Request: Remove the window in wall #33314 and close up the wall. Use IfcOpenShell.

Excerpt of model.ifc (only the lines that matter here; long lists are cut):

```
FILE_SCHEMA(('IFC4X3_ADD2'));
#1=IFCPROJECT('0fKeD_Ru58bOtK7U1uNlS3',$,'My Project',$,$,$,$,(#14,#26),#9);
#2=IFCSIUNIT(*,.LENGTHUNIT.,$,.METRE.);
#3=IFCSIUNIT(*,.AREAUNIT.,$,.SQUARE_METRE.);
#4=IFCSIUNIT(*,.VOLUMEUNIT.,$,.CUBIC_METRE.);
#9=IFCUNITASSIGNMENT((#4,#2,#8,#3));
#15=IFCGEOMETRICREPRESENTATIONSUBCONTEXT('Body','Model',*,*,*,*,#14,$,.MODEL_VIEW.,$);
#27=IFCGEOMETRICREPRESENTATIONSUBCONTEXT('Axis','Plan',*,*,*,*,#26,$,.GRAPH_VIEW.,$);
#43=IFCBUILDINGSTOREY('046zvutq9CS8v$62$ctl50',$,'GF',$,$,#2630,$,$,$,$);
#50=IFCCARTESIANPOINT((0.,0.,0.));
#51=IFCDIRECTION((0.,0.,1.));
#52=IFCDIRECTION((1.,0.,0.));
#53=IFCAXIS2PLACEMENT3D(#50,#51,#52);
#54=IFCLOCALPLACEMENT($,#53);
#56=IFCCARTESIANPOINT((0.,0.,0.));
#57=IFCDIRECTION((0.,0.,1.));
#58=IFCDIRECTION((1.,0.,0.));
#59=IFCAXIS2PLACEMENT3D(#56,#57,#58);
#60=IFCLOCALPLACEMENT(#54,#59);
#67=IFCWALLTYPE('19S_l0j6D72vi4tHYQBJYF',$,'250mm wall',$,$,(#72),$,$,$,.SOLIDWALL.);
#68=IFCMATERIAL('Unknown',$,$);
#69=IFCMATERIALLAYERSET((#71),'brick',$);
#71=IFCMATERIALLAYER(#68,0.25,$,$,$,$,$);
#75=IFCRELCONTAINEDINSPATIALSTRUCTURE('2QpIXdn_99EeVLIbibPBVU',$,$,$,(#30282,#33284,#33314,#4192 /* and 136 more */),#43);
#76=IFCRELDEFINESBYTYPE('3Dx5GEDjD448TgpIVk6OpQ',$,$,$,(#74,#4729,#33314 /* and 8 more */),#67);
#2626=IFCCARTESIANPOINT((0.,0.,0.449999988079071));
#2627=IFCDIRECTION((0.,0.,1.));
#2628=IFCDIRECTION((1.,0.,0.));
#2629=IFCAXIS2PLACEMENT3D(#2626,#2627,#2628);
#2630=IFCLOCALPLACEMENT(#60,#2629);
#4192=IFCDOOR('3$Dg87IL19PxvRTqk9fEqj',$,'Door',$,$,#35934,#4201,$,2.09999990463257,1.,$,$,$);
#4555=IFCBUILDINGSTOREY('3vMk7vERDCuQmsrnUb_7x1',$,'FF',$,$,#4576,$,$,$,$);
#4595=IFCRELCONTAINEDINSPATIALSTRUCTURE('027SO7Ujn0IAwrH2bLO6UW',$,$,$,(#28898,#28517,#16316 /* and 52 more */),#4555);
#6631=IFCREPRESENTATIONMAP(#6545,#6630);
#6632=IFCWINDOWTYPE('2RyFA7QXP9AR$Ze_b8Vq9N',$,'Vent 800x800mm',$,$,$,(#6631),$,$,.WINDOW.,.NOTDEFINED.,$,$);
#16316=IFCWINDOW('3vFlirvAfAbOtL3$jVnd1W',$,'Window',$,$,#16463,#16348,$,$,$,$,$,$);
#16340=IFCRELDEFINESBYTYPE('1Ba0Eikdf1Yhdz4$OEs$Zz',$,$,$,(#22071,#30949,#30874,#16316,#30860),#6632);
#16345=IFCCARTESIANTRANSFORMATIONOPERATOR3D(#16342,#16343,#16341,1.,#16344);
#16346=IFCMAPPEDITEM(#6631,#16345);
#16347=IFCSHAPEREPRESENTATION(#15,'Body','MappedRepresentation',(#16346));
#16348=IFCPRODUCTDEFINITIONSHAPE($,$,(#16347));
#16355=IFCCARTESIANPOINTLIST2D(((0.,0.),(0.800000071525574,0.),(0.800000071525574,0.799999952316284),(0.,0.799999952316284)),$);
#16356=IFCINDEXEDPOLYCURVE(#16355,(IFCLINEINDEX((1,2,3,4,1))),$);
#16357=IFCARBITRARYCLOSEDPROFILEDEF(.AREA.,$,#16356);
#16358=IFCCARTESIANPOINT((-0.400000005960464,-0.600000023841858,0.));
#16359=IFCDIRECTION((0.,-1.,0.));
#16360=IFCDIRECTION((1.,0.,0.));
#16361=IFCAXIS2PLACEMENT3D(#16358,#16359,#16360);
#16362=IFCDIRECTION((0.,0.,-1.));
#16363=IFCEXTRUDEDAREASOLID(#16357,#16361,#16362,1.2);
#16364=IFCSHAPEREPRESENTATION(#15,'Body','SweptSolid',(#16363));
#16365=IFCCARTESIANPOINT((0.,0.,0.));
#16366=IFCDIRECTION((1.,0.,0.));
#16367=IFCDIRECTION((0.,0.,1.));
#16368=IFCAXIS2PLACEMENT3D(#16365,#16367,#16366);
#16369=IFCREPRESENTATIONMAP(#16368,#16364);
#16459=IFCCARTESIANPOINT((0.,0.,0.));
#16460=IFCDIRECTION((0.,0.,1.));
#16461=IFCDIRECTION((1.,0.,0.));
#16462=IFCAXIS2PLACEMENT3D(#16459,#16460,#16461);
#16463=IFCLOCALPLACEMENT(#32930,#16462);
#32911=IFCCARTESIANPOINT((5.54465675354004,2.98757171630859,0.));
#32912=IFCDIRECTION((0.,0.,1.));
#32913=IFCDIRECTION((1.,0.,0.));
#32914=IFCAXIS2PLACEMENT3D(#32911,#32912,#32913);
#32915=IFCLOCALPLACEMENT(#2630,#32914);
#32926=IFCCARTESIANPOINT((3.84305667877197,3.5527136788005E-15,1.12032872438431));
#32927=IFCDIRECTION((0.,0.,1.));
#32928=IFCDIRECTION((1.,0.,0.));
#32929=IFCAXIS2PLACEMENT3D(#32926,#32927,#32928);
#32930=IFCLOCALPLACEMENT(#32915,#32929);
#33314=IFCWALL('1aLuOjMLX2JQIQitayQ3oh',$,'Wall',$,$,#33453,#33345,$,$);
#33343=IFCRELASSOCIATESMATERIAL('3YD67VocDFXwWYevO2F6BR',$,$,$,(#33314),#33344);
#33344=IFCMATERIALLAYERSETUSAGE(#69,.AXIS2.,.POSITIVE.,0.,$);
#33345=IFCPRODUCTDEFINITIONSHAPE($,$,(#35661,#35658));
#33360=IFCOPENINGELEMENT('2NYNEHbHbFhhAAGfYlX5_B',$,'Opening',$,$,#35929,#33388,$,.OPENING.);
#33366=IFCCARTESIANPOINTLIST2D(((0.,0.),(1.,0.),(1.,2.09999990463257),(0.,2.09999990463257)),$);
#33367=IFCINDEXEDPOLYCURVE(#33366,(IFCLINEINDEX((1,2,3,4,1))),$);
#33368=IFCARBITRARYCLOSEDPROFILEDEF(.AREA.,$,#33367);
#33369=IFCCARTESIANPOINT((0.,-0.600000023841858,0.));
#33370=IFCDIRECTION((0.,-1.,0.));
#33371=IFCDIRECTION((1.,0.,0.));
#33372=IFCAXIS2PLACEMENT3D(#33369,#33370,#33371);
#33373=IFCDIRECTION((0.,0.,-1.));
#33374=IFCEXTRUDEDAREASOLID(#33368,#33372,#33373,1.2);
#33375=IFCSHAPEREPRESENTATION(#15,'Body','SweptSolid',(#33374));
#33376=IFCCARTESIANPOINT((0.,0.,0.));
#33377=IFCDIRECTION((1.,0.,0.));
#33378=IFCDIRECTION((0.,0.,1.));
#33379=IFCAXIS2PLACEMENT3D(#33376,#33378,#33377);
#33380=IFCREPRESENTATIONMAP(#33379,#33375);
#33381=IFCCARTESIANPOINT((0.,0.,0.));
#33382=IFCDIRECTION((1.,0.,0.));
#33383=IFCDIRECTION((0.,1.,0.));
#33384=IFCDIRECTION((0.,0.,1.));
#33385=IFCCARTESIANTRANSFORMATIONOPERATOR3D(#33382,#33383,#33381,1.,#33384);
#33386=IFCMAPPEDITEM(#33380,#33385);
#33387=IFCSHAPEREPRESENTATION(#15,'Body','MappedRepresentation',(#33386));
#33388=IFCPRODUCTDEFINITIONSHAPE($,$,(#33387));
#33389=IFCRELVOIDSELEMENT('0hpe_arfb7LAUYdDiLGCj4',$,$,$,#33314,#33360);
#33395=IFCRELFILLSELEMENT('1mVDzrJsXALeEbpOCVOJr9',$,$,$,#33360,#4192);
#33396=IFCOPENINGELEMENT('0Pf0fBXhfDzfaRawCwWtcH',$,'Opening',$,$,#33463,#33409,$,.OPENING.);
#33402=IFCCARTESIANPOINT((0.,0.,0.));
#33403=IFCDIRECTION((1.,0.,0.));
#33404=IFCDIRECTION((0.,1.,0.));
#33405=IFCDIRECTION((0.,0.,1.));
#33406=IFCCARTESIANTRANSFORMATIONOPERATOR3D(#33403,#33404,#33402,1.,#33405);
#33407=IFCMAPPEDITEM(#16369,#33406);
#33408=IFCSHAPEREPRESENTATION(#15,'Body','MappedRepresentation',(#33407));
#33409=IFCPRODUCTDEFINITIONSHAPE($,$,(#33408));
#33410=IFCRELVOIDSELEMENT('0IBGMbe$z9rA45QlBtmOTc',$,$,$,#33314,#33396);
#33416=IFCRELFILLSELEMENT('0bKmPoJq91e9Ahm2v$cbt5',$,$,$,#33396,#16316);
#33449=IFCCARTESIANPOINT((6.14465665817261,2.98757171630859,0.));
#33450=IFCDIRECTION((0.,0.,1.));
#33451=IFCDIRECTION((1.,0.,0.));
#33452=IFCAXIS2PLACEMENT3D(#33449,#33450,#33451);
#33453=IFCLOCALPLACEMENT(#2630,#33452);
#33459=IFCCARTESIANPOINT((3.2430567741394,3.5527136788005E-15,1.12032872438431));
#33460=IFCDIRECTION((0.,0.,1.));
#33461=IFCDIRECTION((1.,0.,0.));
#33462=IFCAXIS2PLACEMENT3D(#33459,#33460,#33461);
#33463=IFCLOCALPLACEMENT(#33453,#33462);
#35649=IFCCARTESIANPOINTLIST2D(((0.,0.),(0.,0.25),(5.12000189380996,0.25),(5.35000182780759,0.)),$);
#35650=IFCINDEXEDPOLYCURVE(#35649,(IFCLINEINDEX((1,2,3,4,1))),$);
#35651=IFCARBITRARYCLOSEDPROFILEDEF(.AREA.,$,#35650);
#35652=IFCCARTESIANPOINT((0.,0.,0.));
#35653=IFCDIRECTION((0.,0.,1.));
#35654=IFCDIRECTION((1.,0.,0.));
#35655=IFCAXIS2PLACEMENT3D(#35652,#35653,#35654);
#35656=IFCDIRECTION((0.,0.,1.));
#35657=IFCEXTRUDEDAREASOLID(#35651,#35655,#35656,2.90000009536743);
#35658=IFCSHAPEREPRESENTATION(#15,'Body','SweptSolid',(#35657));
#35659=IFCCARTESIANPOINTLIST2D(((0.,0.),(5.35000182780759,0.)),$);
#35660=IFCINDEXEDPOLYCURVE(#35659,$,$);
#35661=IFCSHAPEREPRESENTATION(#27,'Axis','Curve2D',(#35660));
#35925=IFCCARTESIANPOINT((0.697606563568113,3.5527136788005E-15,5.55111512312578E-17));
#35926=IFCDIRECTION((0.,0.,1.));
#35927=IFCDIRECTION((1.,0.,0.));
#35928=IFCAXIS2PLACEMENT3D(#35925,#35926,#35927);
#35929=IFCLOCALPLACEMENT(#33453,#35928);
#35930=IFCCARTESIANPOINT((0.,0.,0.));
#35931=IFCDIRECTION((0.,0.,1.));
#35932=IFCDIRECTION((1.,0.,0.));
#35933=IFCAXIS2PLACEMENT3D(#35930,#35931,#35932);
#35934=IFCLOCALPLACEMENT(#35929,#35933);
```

```python
import ifcopenshell
import ifcopenshell.api.feature
import ifcopenshell.api.root
import ifcopenshell.geom
import ifcopenshell.util.shape

model = ifcopenshell.open("model.ifc")
settings = ifcopenshell.geom.settings()


def volume(element):
    """Net volume in cubic metres, openings subtracted."""
    shape = ifcopenshell.geom.create_shape(settings, element)
    return ifcopenshell.util.shape.get_volume(shape.geometry)


window = model.by_guid("3vFlirvAfAbOtL3$jVnd1W")
opening = window.FillsVoids[0].RelatingOpeningElement
wall = opening.VoidsElements[0].RelatingBuildingElement
before = volume(wall)

ifcopenshell.api.root.remove_product(model, product=window)
ifcopenshell.api.feature.remove_feature(model, feature=opening)

after = volume(wall)

print(f"wall volume {before:.3f} -> {after:.3f} m3")

model.write("model_rev.ifc")
```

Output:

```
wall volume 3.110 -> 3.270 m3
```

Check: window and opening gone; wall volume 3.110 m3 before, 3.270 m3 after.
